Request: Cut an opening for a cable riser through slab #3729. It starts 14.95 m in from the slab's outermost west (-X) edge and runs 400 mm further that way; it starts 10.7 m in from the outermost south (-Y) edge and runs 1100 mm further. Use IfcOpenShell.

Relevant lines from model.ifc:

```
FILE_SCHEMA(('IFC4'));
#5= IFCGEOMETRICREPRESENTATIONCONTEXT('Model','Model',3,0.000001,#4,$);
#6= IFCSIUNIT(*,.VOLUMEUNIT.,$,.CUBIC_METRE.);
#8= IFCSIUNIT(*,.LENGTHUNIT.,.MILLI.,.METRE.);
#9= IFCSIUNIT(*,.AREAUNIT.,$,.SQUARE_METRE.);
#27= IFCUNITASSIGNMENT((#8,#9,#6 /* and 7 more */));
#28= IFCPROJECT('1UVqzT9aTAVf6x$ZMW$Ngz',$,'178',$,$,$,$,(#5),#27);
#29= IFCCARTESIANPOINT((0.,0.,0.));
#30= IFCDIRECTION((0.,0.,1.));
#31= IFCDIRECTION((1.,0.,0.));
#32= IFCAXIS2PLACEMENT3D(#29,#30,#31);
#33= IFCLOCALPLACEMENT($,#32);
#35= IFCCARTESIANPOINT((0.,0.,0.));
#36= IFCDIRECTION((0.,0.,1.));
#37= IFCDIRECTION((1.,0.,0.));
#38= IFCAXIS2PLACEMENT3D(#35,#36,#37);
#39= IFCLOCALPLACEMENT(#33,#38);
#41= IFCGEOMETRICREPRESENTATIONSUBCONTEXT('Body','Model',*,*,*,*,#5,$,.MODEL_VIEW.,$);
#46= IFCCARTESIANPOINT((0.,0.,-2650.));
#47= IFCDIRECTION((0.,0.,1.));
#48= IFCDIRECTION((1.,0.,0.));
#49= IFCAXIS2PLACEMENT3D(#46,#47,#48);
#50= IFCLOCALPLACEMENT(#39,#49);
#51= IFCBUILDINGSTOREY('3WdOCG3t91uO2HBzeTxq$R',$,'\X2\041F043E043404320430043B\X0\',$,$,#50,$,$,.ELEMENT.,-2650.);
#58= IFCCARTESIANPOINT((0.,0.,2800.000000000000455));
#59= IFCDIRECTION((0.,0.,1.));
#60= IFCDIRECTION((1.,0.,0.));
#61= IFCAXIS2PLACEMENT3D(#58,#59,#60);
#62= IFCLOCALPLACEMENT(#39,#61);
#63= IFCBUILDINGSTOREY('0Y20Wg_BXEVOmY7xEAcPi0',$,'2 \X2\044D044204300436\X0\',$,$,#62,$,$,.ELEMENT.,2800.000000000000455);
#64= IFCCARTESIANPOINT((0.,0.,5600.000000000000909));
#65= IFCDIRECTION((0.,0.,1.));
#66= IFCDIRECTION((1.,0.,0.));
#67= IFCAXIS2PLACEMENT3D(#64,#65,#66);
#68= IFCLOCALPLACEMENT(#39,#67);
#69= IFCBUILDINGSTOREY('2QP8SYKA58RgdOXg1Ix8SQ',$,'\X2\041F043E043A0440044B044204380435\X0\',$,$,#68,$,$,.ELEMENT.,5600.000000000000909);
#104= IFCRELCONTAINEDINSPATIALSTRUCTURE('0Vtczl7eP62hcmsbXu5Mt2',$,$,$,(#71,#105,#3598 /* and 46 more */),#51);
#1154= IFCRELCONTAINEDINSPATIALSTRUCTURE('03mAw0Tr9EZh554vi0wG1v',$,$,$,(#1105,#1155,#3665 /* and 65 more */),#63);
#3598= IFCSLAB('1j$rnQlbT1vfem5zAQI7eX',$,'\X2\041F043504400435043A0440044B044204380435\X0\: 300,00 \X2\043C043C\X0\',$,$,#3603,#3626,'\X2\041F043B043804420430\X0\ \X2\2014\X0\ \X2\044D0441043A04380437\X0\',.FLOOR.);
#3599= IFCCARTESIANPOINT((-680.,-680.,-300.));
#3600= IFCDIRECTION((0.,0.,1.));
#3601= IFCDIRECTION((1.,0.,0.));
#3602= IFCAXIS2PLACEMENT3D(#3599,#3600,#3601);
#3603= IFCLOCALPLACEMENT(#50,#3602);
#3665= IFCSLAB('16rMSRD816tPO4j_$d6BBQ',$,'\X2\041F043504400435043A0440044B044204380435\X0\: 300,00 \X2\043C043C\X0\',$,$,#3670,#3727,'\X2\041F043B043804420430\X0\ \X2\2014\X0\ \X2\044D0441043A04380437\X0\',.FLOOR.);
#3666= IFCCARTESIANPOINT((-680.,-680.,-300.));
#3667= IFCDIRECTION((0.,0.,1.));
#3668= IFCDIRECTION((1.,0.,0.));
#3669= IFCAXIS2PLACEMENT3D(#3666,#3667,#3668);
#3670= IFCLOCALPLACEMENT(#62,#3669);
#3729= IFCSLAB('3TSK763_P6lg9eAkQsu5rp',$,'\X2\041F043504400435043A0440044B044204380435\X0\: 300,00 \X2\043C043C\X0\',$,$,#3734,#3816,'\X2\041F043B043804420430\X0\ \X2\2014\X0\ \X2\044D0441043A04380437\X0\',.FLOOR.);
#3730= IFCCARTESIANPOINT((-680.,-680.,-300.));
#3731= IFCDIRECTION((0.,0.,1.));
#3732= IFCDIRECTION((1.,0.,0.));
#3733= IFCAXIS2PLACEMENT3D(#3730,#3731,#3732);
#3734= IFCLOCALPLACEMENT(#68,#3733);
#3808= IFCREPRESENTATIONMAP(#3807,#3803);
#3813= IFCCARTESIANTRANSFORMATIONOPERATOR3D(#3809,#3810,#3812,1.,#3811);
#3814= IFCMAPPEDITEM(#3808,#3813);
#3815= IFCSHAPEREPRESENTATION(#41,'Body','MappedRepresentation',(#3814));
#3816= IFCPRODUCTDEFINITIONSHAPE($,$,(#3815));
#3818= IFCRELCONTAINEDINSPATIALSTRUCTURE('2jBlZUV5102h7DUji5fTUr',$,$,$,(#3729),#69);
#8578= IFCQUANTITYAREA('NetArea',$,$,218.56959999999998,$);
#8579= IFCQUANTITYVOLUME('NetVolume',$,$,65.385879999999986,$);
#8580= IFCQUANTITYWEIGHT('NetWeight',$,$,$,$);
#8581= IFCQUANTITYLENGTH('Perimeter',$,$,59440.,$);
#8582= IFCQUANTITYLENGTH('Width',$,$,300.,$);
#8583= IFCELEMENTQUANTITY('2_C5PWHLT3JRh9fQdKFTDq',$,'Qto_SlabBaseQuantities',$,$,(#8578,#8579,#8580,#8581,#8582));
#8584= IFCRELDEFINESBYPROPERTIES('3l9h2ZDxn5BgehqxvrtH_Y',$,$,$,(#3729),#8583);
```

```python
import numpy as np
import ifcopenshell
import ifcopenshell.api.feature
import ifcopenshell.api.geometry
import ifcopenshell.api.pset
import ifcopenshell.api.root
import ifcopenshell.geom
import ifcopenshell.util.element
import ifcopenshell.util.placement
import ifcopenshell.util.representation
import ifcopenshell.util.shape
import ifcopenshell.util.unit

model = ifcopenshell.open("model.ifc")
unit_scale = ifcopenshell.util.unit.calculate_unit_scale(model)
area_scale = ifcopenshell.util.unit.calculate_unit_scale(model, "AREAUNIT")
volume_scale = ifcopenshell.util.unit.calculate_unit_scale(model, "VOLUMEUNIT")
settings = ifcopenshell.geom.settings()


def volume(element):
    """Net volume in cubic metres, openings subtracted."""
    shape = ifcopenshell.geom.create_shape(settings, element)
    return ifcopenshell.util.shape.get_volume(shape.geometry)


slab = model.by_id(3729)
before = volume(slab)

# Extent in the slab's own axes, in metres. The edges named are its -X and -Y sides.
slab_shape = ifcopenshell.geom.create_shape(settings, slab)
vertices = ifcopenshell.util.shape.get_vertices(slab_shape.geometry)
x_min, y_min, bottom = vertices.min(axis=0)
top = vertices[:, 2].max()

opening = ifcopenshell.api.root.create_entity(model, ifc_class="IfcOpeningElement", name="Cable riser opening", predefined_type="OPENING")
context = ifcopenshell.util.representation.get_context(model, "Model", "Body", "MODEL_VIEW")
width, depth = 0.4, 1.1
outline = [(0.0, 0.0), (width, 0.0), (width, depth), (0.0, depth), (0.0, 0.0)]
# Overshoot both faces by 50 mm so the cut is clean.
shape = ifcopenshell.api.geometry.add_slab_representation(
    model, context=context, depth=top - bottom + 0.1, polyline=outline
)
ifcopenshell.api.geometry.assign_representation(model, product=opening, representation=shape)

matrix = ifcopenshell.util.placement.get_local_placement(slab.ObjectPlacement)
matrix[:, 3] = matrix @ np.append(np.array([x_min + 14.95, y_min + 10.7, bottom - 0.05]) / unit_scale, 1.0)
ifcopenshell.api.geometry.edit_object_placement(model, product=opening, matrix=matrix, is_si=False)
ifcopenshell.api.feature.add_feature(model, feature=opening, element=slab)

after = volume(slab)

# Update the slab's stored quantities.
qto = model.by_id(ifcopenshell.util.element.get_pset(slab, "Qto_SlabBaseQuantities", should_inherit=False)["id"])
ifcopenshell.api.pset.edit_qto(model, qto=qto, properties={
    "NetArea": after / (top - bottom) / area_scale,
    "NetVolume": after / volume_scale,
})

print(f"slab volume {before:.3f} -> {after:.3f} m3")

model.write("model_v2.ifc")
```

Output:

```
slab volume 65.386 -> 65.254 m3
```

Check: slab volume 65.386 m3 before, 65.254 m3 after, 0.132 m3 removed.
